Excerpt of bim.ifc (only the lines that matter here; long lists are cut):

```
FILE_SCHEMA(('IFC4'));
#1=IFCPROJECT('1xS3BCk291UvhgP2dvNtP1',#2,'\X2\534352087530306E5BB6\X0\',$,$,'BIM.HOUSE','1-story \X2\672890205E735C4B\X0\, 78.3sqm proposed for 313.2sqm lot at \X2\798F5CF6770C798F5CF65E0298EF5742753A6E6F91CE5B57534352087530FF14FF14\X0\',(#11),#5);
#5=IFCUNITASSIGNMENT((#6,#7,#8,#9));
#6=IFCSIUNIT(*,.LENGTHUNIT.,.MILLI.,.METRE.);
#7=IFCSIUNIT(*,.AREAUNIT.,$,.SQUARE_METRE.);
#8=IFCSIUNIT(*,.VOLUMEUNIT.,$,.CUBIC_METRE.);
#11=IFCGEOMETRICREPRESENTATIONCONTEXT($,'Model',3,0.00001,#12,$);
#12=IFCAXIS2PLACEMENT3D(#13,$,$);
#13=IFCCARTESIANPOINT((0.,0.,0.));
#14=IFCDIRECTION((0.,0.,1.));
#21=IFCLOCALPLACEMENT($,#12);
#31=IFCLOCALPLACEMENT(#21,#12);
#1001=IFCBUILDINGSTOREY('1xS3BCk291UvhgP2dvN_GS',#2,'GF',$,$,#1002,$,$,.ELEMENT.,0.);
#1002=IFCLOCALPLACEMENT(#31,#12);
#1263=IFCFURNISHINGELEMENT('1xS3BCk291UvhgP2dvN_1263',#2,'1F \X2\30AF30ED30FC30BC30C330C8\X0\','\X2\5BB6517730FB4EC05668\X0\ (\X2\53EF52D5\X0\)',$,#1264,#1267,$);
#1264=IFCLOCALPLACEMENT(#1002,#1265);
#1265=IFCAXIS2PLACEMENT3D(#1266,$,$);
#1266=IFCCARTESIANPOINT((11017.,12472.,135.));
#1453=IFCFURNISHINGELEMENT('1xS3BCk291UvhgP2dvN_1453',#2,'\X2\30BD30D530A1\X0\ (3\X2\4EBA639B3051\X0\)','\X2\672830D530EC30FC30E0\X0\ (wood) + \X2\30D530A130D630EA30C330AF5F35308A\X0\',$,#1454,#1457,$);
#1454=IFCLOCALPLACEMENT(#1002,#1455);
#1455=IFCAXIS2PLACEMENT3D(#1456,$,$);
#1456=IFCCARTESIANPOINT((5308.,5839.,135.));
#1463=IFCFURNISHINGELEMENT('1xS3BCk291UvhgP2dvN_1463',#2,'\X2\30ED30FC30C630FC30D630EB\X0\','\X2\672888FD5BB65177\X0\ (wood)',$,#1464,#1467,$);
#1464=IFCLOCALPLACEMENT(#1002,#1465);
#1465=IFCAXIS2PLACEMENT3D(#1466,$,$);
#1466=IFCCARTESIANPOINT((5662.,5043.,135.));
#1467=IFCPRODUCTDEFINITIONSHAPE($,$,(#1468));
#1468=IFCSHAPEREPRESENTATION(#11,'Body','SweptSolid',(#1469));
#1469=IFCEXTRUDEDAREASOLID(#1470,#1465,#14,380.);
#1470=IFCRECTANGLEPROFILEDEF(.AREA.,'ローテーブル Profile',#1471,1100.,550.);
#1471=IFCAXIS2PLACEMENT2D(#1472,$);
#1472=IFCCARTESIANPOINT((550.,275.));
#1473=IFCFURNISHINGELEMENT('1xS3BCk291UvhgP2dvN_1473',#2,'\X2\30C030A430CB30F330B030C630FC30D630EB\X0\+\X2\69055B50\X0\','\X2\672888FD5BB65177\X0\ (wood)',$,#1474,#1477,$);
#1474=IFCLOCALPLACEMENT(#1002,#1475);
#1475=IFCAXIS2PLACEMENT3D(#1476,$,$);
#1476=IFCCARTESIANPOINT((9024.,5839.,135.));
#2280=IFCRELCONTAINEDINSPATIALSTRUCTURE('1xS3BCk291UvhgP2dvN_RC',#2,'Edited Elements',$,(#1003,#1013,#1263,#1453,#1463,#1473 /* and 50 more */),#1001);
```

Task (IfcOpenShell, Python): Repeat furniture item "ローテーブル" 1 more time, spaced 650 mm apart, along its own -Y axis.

```python
import ifcopenshell
import ifcopenshell.api.geometry
import ifcopenshell.api.root
import ifcopenshell.util.element
import ifcopenshell.util.placement
import ifcopenshell.util.unit

model = ifcopenshell.open("bim.ifc")
unit_scale = ifcopenshell.util.unit.calculate_unit_scale(model)


def reuse_history(source, copy):
    """copy_class also copies each property set's owner history, people and application; keep the originals."""
    for rel in copy.IsDefinedBy:
        if rel.is_a("IfcRelDefinesByProperties") and (history := rel.RelatingPropertyDefinition.OwnerHistory):
            rel.RelatingPropertyDefinition.OwnerHistory = source.OwnerHistory
            ifcopenshell.util.element.remove_deep2(model, history)


source = model.by_guid("1xS3BCk291UvhgP2dvN_1463")
base = ifcopenshell.util.placement.get_local_placement(source.ObjectPlacement)
step = -base[:3, 1] * 0.65 / unit_scale

for i in range(1, 2):
    copy = ifcopenshell.api.root.copy_class(model, product=source)
    copy.Representation = ifcopenshell.util.element.copy_deep(
        model, source.Representation, exclude=["IfcGeometricRepresentationContext", "IfcRepresentationMap"]
    )
    reuse_history(source, copy)
    matrix = base.copy()
    matrix[:3, 3] += i * step
    print("added at", matrix[:3, 3].round(3) + 0.0)
    ifcopenshell.api.geometry.edit_object_placement(model, product=copy, matrix=matrix, is_si=False)

model.write("bim_v2.ifc")
```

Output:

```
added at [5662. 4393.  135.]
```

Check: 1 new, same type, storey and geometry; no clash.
